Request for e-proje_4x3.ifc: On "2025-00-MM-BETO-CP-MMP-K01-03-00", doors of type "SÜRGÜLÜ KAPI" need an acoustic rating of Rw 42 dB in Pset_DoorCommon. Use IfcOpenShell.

First a look at what the model holds.

```python
import ifcopenshell
import ifcopenshell.util.element

model = ifcopenshell.open("e-proje_4x3.ifc")
print(model.schema)
storey = next(s for s in model.by_type("IfcBuildingStorey") if s.Name == "2025-00-MM-BETO-CP-MMP-K01-03-00")
doors = [e for e in ifcopenshell.util.element.get_decomposition(storey) if e.is_a("IfcDoor")]
seen = {}
for e in doors:
    element_type = ifcopenshell.util.element.get_type(e)
    key = (element_type.Name if element_type != e and element_type else None, ifcopenshell.util.element.get_pset(e, "Pset_DoorCommon", "AcousticRating"))
    seen[key] = seen.get(key, 0) + 1
for (name, value), count in sorted(seen.items(), key=str):
    print(count, "x", name, "|", value)
```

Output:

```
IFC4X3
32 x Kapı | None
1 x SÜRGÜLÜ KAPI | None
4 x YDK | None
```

```python
import ifcopenshell
import ifcopenshell.api.pset
import ifcopenshell.util.element

model = ifcopenshell.open("e-proje_4x3.ifc")

storey = next(s for s in model.by_type("IfcBuildingStorey") if s.Name == "2025-00-MM-BETO-CP-MMP-K01-03-00")
doors = [e for e in ifcopenshell.util.element.get_decomposition(storey) if e.is_a("IfcDoor")]

count = 0
for e in doors:
    element_type = ifcopenshell.util.element.get_type(e)
    if element_type in (None, e) or element_type.Name != "SÜRGÜLÜ KAPI":
        continue
    # add_pset returns the element's existing set when there is one.
    pset = ifcopenshell.api.pset.add_pset(model, product=e, name="Pset_DoorCommon")
    ifcopenshell.api.pset.edit_pset(model, pset=pset, properties={"AcousticRating": "Rw 42 dB"})
    count += 1

print(count, "doors updated")

model.write("e-proje_4x3_edited.ifc")
```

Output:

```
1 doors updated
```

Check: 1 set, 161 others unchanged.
